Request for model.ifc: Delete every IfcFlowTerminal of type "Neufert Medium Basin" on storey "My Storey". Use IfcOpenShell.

First a look at what the model holds.

```python
import ifcopenshell
import ifcopenshell.util.element

model = ifcopenshell.open("model.ifc")
print(model.schema)
storey = next(s for s in model.by_type("IfcBuildingStorey") if s.Name == "My Storey")
terminals = [e for e in ifcopenshell.util.element.get_decomposition(storey) if e.is_a("IfcFlowTerminal")]
seen = {}
for e in terminals:
    element_type = ifcopenshell.util.element.get_type(e)
    name = element_type.Name if element_type not in (None, e) else None
    seen[name] = seen.get(name, 0) + 1
for name, count in sorted(seen.items(), key=str):
    print(count, "x", name)
```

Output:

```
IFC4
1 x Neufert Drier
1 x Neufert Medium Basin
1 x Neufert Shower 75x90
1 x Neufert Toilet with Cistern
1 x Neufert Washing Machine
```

```python
import ifcopenshell
import ifcopenshell.api.root
import ifcopenshell.util.element

model = ifcopenshell.open("model.ifc")

storey = next(s for s in model.by_type("IfcBuildingStorey") if s.Name == "My Storey")
terminals = [e for e in ifcopenshell.util.element.get_decomposition(storey) if e.is_a("IfcFlowTerminal")]
targets = [e for e in terminals if (t := ifcopenshell.util.element.get_type(e)) not in (None, e) and t.Name == "Neufert Medium Basin"]

for e in targets:
    ifcopenshell.api.root.remove_product(model, product=e)
print(len(targets), "removed")

model.write("model_v2.ifc")
```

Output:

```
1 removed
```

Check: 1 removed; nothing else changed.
